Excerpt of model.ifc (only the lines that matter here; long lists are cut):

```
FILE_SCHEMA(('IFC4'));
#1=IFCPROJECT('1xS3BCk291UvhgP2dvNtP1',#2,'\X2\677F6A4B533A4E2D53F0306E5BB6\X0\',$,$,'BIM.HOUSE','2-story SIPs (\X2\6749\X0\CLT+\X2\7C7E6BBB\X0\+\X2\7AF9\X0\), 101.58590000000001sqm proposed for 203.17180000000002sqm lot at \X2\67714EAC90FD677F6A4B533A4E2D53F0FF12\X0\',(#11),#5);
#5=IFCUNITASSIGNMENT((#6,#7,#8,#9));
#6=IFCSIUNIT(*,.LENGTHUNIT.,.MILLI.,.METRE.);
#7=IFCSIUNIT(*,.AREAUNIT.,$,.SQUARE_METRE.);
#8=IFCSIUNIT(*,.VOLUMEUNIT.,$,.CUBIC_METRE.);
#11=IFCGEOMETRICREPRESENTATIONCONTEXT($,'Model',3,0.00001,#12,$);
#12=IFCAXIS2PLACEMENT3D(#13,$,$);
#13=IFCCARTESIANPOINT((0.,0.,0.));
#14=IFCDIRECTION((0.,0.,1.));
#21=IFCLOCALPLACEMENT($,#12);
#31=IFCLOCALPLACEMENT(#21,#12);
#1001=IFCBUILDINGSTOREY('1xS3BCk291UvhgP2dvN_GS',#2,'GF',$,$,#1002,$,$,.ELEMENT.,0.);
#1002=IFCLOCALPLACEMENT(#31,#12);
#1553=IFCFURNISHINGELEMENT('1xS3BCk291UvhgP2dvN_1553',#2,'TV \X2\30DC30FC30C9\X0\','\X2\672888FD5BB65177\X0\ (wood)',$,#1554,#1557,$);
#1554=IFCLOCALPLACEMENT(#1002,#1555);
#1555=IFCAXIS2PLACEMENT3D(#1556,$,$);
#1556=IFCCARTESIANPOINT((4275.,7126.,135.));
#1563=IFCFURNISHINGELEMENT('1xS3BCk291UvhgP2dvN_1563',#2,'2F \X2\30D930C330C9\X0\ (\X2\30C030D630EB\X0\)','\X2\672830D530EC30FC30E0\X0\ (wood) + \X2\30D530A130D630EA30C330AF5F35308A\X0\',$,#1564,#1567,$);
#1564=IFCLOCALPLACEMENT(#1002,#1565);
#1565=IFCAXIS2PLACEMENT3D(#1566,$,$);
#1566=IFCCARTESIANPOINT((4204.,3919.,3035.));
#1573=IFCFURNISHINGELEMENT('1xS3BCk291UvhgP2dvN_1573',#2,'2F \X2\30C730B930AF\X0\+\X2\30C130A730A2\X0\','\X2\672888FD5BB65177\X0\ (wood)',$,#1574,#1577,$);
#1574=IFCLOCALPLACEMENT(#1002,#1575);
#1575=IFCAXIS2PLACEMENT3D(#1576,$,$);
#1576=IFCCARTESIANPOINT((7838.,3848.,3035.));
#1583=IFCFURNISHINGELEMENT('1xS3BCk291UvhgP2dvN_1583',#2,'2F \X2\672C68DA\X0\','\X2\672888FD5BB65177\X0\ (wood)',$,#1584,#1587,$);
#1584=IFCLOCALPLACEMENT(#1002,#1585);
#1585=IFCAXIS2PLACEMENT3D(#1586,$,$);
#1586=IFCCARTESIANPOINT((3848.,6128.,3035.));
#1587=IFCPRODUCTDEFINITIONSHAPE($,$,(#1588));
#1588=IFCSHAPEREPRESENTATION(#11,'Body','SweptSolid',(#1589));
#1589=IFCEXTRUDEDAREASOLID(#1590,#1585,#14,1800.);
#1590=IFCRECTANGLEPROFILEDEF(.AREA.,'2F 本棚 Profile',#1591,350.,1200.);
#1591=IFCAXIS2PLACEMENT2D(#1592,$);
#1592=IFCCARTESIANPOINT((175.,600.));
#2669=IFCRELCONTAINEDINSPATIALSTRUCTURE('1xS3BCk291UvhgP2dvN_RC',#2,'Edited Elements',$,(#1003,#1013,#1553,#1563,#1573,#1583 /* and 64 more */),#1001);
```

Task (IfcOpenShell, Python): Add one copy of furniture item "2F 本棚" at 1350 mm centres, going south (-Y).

```python
import numpy as np
import ifcopenshell
import ifcopenshell.api.geometry
import ifcopenshell.api.root
import ifcopenshell.util.element
import ifcopenshell.util.placement
import ifcopenshell.util.unit

model = ifcopenshell.open("model.ifc")
unit_scale = ifcopenshell.util.unit.calculate_unit_scale(model)


def reuse_history(source, copy):
    """copy_class also copies each property set's owner history, people and application; keep the originals."""
    for rel in copy.IsDefinedBy:
        if rel.is_a("IfcRelDefinesByProperties") and (history := rel.RelatingPropertyDefinition.OwnerHistory):
            rel.RelatingPropertyDefinition.OwnerHistory = source.OwnerHistory
            ifcopenshell.util.element.remove_deep2(model, history)


source = model.by_guid("1xS3BCk291UvhgP2dvN_1583")
base = ifcopenshell.util.placement.get_local_placement(source.ObjectPlacement)
step = np.array([0.0, -1.0, 0.0]) * 1.35 / unit_scale

for i in range(1, 2):
    copy = ifcopenshell.api.root.copy_class(model, product=source)
    copy.Representation = ifcopenshell.util.element.copy_deep(
        model, source.Representation, exclude=["IfcGeometricRepresentationContext", "IfcRepresentationMap"]
    )
    reuse_history(source, copy)
    matrix = base.copy()
    matrix[:3, 3] += i * step
    print("added at", matrix[:3, 3].round(3) + 0.0)
    ifcopenshell.api.geometry.edit_object_placement(model, product=copy, matrix=matrix, is_si=False)

model.write("model_edited.ifc")
```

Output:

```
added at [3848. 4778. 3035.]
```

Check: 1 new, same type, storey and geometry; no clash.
